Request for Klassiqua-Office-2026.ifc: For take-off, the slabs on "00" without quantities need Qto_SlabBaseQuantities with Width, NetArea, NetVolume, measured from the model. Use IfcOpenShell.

First a look at what the model holds.

```python
import ifcopenshell
import ifcopenshell.util.element
import ifcopenshell.util.unit

model = ifcopenshell.open("Klassiqua-Office-2026.ifc")
print(model.schema)
for unit_type in ("LENGTHUNIT", "AREAUNIT", "VOLUMEUNIT"):
    print(unit_type, ifcopenshell.util.unit.calculate_unit_scale(model, unit_type))
storey = next(s for s in model.by_type("IfcBuildingStorey") if s.Name == "00")
slabs = [e for e in ifcopenshell.util.element.get_decomposition(storey) if e.is_a("IfcSlab")]
for e in sorted(slabs, key=lambda e: e.id()):
    print(e.id(), e.is_a(), e.Name, list(ifcopenshell.util.element.get_psets(e, qtos_only=True)), sep=" | ")
```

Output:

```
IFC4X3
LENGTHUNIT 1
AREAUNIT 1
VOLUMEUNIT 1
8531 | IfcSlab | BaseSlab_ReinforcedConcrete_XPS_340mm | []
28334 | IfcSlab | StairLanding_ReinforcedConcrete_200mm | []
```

```python
import ifcopenshell
import ifcopenshell.api.pset
import ifcopenshell.geom
import ifcopenshell.util.element
import ifcopenshell.util.shape
import ifcopenshell.util.unit

model = ifcopenshell.open("Klassiqua-Office-2026.ifc")
unit_scale = ifcopenshell.util.unit.calculate_unit_scale(model)
area_scale = ifcopenshell.util.unit.calculate_unit_scale(model, "AREAUNIT")
volume_scale = ifcopenshell.util.unit.calculate_unit_scale(model, "VOLUMEUNIT")
settings = ifcopenshell.geom.settings()

storey = next(s for s in model.by_type("IfcBuildingStorey") if s.Name == "00")
slabs = [e for e in ifcopenshell.util.element.get_decomposition(storey) if e.is_a("IfcSlab")]

for e in sorted(slabs, key=lambda e: e.id()):
    if ifcopenshell.util.element.get_psets(e, qtos_only=True, should_inherit=False):
        continue
    # Geometry comes back in metres, in the element's own axes.
    shape = ifcopenshell.geom.create_shape(settings, e)
    values = {
        "Width": ifcopenshell.util.shape.get_z(shape.geometry) / unit_scale,
        "NetArea": ifcopenshell.util.shape.get_footprint_area(shape.geometry) / area_scale,
        "NetVolume": ifcopenshell.util.shape.get_volume(shape.geometry) / volume_scale,
    }
    qto = ifcopenshell.api.pset.add_qto(model, product=e, name="Qto_SlabBaseQuantities")
    ifcopenshell.api.pset.edit_qto(model, qto=qto, properties=values)
    print(e.id(), {k: round(v, 3) for k, v in values.items()})

model.write("Klassiqua-Office-2026_updated.ifc")
```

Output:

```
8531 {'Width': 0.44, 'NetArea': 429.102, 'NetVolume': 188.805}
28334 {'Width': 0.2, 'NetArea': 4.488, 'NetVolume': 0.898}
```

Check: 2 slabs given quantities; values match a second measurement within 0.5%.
